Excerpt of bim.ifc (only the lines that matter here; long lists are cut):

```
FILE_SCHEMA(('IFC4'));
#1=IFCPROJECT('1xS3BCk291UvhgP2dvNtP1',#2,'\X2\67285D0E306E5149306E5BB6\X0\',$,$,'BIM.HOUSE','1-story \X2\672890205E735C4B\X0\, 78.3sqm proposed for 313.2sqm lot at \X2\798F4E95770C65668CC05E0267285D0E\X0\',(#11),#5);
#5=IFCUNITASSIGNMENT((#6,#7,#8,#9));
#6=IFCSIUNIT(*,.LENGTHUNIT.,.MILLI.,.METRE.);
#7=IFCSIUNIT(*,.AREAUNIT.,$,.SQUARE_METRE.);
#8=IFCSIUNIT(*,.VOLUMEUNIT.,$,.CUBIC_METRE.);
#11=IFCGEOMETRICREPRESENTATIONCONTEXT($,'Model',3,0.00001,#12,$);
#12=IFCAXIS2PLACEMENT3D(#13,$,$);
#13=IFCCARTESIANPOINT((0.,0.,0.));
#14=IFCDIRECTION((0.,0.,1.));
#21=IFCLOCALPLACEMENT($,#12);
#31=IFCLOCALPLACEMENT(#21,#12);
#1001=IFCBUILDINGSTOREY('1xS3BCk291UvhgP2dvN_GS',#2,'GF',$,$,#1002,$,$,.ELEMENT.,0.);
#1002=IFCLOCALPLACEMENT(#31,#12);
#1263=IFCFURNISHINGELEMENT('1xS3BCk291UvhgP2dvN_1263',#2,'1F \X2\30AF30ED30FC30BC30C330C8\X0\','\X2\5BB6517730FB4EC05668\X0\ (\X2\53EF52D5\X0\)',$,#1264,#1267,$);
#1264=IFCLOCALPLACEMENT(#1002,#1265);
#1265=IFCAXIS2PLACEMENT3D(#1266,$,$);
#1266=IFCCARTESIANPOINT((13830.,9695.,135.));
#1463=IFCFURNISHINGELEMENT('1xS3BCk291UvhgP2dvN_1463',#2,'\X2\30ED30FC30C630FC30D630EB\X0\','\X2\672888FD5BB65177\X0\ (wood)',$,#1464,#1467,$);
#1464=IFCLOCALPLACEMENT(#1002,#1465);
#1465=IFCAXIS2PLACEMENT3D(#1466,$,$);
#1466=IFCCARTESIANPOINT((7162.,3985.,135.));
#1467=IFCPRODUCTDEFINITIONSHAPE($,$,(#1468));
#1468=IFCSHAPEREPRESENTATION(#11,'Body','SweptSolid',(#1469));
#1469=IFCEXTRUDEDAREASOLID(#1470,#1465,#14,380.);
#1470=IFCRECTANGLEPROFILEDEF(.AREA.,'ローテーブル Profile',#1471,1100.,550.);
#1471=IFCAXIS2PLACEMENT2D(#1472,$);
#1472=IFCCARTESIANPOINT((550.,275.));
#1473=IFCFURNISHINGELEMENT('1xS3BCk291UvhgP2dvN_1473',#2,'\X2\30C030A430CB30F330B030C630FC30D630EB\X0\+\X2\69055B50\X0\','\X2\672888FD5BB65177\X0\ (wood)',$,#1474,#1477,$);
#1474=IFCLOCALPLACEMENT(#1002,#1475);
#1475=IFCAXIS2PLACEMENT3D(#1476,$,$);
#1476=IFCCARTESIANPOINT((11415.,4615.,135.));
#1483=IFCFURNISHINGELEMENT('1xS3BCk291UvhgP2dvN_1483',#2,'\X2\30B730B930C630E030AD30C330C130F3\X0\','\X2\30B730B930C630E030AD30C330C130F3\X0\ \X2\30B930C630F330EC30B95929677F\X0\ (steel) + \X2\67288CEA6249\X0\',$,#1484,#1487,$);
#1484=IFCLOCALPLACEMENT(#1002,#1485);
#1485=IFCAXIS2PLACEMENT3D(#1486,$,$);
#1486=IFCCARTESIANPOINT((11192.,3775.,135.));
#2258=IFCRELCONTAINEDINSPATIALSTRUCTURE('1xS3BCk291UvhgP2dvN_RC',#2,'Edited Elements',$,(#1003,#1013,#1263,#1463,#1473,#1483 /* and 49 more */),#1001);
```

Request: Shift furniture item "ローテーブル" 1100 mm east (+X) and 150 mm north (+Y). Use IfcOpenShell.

```python
import ifcopenshell
import ifcopenshell.api.geometry
import ifcopenshell.util.placement
import ifcopenshell.util.unit

model = ifcopenshell.open("bim.ifc")
unit_scale = ifcopenshell.util.unit.calculate_unit_scale(model)

item = model.by_id(1463)
matrix = ifcopenshell.util.placement.get_local_placement(item.ObjectPlacement)
matrix[0, 3] += 1.1 / unit_scale
matrix[1, 3] += 0.15 / unit_scale
ifcopenshell.api.geometry.edit_object_placement(model, product=item, matrix=matrix, is_si=False)

print(ifcopenshell.util.placement.get_local_placement(item.ObjectPlacement).round(3) + 0.0)

model.write("bim-out.ifc")
```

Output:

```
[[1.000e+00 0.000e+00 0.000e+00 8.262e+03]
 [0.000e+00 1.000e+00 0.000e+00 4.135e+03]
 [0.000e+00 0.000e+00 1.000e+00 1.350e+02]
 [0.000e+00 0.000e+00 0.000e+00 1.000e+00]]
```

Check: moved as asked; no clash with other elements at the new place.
